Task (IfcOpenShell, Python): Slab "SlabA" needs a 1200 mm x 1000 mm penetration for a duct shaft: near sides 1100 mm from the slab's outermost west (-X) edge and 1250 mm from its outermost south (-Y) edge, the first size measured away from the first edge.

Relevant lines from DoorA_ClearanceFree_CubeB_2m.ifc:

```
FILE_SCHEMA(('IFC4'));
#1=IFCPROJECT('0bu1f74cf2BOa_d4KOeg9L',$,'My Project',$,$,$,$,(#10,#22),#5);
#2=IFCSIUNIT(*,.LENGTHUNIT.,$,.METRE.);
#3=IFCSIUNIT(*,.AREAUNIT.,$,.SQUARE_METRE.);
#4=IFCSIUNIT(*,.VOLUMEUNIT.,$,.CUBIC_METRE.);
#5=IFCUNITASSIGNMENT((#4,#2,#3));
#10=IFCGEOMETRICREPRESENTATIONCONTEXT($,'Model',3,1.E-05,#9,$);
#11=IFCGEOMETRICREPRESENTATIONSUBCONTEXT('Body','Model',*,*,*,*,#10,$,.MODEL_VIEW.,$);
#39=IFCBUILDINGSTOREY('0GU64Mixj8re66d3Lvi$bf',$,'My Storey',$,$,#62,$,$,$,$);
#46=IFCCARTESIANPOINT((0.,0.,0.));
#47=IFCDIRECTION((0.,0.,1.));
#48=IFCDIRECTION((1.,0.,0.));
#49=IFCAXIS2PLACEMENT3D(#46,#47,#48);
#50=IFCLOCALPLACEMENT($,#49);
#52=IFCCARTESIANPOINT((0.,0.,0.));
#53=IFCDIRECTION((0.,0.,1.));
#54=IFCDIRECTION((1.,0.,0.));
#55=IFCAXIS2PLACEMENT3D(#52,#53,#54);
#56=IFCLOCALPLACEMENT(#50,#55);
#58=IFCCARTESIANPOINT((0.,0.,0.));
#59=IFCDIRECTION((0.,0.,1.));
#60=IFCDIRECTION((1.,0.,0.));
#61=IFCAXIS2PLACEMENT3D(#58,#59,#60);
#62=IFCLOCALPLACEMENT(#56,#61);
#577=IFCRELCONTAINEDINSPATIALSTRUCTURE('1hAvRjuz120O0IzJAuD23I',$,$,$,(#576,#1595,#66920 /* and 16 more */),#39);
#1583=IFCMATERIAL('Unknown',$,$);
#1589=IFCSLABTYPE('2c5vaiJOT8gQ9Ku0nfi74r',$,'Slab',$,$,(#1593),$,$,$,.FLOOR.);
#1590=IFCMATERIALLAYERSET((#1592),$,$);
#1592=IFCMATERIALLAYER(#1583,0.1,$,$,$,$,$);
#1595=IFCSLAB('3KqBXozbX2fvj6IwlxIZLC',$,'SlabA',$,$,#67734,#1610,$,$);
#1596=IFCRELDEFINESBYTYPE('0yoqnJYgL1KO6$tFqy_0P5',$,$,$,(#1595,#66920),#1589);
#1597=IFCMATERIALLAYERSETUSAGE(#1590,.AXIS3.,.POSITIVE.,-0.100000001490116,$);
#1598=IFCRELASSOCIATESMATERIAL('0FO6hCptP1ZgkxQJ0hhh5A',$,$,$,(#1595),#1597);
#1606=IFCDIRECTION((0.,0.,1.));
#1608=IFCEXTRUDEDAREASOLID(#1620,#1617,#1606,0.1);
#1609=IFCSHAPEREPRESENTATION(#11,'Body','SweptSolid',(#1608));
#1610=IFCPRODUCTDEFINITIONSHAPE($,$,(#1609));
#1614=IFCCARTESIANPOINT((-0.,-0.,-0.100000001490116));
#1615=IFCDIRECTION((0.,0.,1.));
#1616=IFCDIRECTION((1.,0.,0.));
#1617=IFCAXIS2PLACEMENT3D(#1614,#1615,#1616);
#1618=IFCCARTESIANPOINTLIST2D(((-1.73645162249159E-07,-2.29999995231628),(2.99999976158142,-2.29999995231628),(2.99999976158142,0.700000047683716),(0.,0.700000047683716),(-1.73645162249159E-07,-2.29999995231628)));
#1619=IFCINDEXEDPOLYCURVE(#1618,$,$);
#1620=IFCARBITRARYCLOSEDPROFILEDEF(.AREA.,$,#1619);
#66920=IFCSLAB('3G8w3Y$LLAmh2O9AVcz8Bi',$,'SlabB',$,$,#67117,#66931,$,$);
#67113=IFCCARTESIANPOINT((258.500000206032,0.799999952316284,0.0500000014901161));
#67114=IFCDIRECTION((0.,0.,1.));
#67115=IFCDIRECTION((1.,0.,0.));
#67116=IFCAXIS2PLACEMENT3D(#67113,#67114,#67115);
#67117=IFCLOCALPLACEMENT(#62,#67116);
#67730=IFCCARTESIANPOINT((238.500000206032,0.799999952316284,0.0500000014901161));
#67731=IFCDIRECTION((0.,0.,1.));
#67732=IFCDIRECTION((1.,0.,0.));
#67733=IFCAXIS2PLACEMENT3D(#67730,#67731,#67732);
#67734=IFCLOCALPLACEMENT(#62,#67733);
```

```python
import numpy as np
import ifcopenshell
import ifcopenshell.api.feature
import ifcopenshell.api.geometry
import ifcopenshell.api.root
import ifcopenshell.geom
import ifcopenshell.util.placement
import ifcopenshell.util.representation
import ifcopenshell.util.shape
import ifcopenshell.util.unit

model = ifcopenshell.open("DoorA_ClearanceFree_CubeB_2m.ifc")
unit_scale = ifcopenshell.util.unit.calculate_unit_scale(model)
settings = ifcopenshell.geom.settings()


def volume(element):
    """Net volume in cubic metres, openings subtracted."""
    shape = ifcopenshell.geom.create_shape(settings, element)
    return ifcopenshell.util.shape.get_volume(shape.geometry)


slab = model.by_guid("3KqBXozbX2fvj6IwlxIZLC")
before = volume(slab)

# Extent in the slab's own axes, in metres. The edges named are its -X and -Y sides.
slab_shape = ifcopenshell.geom.create_shape(settings, slab)
vertices = ifcopenshell.util.shape.get_vertices(slab_shape.geometry)
x_min, y_min, bottom = vertices.min(axis=0)
top = vertices[:, 2].max()

opening = ifcopenshell.api.root.create_entity(model, ifc_class="IfcOpeningElement", name="Duct shaft opening", predefined_type="OPENING")
context = ifcopenshell.util.representation.get_context(model, "Model", "Body", "MODEL_VIEW")
width, depth = 1.2, 1
outline = [(0.0, 0.0), (width, 0.0), (width, depth), (0.0, depth), (0.0, 0.0)]
# Overshoot both faces by 50 mm so the cut is clean.
shape = ifcopenshell.api.geometry.add_slab_representation(
    model, context=context, depth=top - bottom + 0.1, polyline=outline
)
ifcopenshell.api.geometry.assign_representation(model, product=opening, representation=shape)

matrix = ifcopenshell.util.placement.get_local_placement(slab.ObjectPlacement)
matrix[:, 3] = matrix @ np.append(np.array([x_min + 1.1, y_min + 1.25, bottom - 0.05]) / unit_scale, 1.0)
ifcopenshell.api.geometry.edit_object_placement(model, product=opening, matrix=matrix, is_si=False)
ifcopenshell.api.feature.add_feature(model, feature=opening, element=slab)

after = volume(slab)

print(f"slab volume {before:.3f} -> {after:.3f} m3")

model.write("DoorA_ClearanceFree_CubeB_2m_v2.ifc")
```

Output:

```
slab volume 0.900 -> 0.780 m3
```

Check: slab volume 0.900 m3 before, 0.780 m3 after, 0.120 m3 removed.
